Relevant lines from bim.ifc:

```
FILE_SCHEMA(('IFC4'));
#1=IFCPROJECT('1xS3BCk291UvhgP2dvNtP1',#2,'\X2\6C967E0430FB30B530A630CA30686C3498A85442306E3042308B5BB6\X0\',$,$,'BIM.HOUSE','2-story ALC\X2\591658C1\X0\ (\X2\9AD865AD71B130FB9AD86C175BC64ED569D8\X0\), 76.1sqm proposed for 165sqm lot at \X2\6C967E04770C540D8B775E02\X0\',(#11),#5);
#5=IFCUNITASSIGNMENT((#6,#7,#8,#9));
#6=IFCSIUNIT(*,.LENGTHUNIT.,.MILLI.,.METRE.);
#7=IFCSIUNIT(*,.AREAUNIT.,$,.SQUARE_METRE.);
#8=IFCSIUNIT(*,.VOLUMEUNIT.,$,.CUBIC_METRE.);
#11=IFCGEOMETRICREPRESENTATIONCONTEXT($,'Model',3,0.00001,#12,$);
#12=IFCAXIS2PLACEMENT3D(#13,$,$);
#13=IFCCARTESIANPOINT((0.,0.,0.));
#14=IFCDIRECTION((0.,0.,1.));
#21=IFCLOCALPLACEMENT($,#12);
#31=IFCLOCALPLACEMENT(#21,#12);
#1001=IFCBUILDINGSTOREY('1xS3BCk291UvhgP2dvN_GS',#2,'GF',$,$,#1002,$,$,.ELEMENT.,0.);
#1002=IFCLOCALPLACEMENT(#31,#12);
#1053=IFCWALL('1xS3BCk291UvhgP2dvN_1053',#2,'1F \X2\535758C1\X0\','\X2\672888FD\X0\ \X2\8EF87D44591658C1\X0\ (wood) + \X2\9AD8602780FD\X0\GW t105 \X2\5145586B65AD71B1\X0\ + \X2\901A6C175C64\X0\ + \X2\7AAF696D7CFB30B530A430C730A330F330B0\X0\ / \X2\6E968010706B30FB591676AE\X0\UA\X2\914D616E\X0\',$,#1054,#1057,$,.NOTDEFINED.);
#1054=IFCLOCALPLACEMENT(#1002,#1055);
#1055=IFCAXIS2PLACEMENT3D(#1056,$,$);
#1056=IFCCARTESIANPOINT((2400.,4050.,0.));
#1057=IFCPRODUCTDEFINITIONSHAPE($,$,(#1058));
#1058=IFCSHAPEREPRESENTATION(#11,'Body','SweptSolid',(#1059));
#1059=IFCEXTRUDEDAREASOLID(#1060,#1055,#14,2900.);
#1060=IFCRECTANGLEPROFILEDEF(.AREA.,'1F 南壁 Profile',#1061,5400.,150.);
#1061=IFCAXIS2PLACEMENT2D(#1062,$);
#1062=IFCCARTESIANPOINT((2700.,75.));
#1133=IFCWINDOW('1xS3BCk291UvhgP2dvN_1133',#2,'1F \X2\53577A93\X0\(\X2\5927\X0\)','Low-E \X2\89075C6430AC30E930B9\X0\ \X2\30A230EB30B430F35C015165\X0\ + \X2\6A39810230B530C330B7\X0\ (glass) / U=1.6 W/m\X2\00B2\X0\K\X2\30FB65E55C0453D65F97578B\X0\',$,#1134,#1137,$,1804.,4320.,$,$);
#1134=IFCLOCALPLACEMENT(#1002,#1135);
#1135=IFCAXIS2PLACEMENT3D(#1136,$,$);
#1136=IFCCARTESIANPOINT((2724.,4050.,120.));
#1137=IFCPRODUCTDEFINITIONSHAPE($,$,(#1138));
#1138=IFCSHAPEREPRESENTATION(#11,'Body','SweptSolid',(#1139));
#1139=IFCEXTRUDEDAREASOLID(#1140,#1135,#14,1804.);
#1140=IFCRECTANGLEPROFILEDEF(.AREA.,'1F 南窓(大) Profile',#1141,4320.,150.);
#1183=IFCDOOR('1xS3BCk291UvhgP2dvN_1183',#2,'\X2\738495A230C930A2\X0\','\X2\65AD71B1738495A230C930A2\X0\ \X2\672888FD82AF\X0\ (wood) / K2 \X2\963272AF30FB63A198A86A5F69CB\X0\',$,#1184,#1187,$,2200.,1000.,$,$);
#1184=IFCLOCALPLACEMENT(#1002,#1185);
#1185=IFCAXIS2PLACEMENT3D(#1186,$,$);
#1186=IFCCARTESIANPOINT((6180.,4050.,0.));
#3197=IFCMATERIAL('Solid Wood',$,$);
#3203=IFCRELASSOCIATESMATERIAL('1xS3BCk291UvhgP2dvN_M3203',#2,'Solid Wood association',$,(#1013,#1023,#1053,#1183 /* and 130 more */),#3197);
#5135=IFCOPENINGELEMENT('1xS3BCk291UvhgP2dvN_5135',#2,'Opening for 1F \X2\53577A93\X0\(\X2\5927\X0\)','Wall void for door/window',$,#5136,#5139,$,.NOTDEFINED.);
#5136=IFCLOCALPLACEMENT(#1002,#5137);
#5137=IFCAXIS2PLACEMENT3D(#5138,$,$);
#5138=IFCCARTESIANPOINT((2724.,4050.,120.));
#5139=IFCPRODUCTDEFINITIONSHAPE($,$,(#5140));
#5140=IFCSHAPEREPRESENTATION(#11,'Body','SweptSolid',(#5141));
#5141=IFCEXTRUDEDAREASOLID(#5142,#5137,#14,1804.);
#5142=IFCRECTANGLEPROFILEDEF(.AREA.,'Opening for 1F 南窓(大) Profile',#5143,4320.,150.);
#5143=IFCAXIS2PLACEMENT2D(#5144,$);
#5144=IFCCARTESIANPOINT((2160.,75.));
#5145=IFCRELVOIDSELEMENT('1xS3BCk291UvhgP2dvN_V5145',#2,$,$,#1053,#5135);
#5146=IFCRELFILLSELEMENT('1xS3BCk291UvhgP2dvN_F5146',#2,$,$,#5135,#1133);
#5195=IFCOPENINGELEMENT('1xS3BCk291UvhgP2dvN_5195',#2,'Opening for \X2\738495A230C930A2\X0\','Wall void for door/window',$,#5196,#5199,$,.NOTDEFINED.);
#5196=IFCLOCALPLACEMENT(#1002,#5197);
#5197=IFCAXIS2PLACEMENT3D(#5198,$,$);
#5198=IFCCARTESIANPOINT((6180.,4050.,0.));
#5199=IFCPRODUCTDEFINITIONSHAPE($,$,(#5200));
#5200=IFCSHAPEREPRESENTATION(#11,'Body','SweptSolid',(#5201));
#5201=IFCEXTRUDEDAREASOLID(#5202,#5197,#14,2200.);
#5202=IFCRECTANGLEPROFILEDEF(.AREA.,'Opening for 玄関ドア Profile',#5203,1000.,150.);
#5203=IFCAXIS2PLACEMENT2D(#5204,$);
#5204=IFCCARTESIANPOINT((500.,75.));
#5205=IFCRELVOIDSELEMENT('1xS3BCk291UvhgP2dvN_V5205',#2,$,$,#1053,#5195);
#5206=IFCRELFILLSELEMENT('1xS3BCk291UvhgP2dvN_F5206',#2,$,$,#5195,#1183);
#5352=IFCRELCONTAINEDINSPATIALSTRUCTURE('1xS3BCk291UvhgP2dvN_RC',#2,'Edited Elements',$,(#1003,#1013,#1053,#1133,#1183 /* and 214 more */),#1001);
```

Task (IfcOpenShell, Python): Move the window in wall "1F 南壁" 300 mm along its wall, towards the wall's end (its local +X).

```python
import ifcopenshell
import ifcopenshell.api.geometry
import ifcopenshell.util.placement
import ifcopenshell.util.unit

model = ifcopenshell.open("bim.ifc")
unit_scale = ifcopenshell.util.unit.calculate_unit_scale(model)

window = model.by_guid("1xS3BCk291UvhgP2dvN_1133")
opening = window.FillsVoids[0].RelatingOpeningElement
wall = opening.VoidsElements[0].RelatingBuildingElement

wall_matrix = ifcopenshell.util.placement.get_local_placement(wall.ObjectPlacement)
shift = wall_matrix[:3, 0] * 0.3 / unit_scale
before = ifcopenshell.util.placement.get_local_placement(window.ObjectPlacement)[:3, 3].copy()

# The window is not placed relative to its opening, so move both.
for product in (opening, window):
    matrix = ifcopenshell.util.placement.get_local_placement(product.ObjectPlacement)
    matrix[:3, 3] += shift
    ifcopenshell.api.geometry.edit_object_placement(model, product=product, matrix=matrix, is_si=False)

after = ifcopenshell.util.placement.get_local_placement(window.ObjectPlacement)[:3, 3]
print("window moved by", (after - before).round(3) + 0.0)

model.write("bim-out.ifc")
```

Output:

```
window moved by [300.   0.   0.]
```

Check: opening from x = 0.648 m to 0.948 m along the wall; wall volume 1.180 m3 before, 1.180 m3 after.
